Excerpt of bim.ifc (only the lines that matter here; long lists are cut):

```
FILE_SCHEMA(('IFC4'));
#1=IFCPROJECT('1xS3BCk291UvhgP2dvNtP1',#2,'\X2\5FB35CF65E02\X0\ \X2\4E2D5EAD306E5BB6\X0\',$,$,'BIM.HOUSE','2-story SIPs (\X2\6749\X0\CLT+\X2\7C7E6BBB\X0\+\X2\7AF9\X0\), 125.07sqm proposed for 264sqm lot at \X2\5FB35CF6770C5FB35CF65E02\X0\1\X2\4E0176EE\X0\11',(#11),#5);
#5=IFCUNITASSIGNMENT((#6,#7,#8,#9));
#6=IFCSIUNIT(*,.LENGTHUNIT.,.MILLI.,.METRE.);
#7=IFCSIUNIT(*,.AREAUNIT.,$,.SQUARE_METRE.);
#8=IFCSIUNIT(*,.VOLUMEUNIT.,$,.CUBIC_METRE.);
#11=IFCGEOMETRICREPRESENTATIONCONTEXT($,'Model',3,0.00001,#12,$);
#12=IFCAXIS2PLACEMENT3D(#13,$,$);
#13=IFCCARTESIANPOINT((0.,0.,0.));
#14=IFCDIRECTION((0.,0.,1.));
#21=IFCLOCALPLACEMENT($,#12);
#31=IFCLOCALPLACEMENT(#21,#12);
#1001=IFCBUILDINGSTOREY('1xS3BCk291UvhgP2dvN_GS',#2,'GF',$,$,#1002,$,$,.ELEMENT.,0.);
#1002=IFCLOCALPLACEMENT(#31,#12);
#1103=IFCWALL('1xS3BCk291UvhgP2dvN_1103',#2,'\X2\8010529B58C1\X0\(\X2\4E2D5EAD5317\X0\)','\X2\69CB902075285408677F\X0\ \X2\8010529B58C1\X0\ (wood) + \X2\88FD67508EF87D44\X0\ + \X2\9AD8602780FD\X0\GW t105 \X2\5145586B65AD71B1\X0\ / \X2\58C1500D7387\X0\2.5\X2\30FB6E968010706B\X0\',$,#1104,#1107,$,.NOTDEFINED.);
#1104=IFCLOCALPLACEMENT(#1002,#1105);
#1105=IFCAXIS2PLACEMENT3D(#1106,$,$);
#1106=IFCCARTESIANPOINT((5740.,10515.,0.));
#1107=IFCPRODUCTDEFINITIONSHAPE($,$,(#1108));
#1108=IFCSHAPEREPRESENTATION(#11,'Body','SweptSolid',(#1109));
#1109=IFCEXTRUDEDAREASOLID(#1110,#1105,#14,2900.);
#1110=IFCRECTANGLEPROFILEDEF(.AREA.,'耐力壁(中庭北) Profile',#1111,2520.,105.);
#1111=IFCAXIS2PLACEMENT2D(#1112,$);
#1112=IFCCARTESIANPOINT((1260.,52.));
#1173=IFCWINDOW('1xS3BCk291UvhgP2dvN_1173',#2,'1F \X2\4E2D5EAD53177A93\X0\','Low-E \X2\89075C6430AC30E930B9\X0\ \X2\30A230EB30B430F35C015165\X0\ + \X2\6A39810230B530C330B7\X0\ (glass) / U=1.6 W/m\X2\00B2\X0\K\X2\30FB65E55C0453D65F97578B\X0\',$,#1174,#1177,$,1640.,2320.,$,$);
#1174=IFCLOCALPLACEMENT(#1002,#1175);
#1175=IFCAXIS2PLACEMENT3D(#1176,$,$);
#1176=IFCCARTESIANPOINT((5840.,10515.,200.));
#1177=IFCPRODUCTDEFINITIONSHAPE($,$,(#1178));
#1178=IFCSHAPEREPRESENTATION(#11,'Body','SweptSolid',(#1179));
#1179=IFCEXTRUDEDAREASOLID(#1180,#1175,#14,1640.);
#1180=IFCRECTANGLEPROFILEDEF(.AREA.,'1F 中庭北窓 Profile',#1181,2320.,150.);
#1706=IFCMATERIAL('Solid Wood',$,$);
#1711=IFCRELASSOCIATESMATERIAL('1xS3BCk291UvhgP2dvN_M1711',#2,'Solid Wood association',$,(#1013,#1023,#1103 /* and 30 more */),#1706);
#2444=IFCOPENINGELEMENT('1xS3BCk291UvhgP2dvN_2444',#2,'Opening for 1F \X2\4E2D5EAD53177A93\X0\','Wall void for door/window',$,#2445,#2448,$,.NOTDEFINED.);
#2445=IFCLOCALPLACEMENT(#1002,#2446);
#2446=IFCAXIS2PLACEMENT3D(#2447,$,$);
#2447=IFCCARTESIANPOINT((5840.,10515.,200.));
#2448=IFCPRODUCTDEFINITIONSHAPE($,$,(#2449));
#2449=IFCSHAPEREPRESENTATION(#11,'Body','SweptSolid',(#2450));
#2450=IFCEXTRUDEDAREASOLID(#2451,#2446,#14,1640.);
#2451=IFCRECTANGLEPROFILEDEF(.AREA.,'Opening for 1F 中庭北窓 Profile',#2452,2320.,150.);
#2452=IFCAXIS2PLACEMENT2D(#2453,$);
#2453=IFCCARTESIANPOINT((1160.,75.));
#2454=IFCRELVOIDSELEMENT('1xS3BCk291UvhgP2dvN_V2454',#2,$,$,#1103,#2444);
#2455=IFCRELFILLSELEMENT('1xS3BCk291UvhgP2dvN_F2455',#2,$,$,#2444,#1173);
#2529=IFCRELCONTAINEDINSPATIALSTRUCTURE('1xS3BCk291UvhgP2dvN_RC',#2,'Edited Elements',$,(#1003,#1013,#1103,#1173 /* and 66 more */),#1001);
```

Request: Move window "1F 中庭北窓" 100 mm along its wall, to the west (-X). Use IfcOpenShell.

```python
import ifcopenshell
import ifcopenshell.api.geometry
import ifcopenshell.util.placement
import ifcopenshell.util.unit

model = ifcopenshell.open("bim.ifc")
unit_scale = ifcopenshell.util.unit.calculate_unit_scale(model)

window = model.by_guid("1xS3BCk291UvhgP2dvN_1173")
opening = window.FillsVoids[0].RelatingOpeningElement
wall = opening.VoidsElements[0].RelatingBuildingElement

wall_matrix = ifcopenshell.util.placement.get_local_placement(wall.ObjectPlacement)
shift = wall_matrix[:3, 0] * -0.1 / unit_scale
before = ifcopenshell.util.placement.get_local_placement(window.ObjectPlacement)[:3, 3].copy()

# The window is not placed relative to its opening, so move both.
for product in (opening, window):
    matrix = ifcopenshell.util.placement.get_local_placement(product.ObjectPlacement)
    matrix[:3, 3] += shift
    ifcopenshell.api.geometry.edit_object_placement(model, product=product, matrix=matrix, is_si=False)

after = ifcopenshell.util.placement.get_local_placement(window.ObjectPlacement)[:3, 3]
print("window moved by", (after - before).round(3) + 0.0)

model.write("bim-out.ifc")
```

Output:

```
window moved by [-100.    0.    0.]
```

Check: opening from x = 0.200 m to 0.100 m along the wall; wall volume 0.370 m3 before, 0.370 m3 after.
